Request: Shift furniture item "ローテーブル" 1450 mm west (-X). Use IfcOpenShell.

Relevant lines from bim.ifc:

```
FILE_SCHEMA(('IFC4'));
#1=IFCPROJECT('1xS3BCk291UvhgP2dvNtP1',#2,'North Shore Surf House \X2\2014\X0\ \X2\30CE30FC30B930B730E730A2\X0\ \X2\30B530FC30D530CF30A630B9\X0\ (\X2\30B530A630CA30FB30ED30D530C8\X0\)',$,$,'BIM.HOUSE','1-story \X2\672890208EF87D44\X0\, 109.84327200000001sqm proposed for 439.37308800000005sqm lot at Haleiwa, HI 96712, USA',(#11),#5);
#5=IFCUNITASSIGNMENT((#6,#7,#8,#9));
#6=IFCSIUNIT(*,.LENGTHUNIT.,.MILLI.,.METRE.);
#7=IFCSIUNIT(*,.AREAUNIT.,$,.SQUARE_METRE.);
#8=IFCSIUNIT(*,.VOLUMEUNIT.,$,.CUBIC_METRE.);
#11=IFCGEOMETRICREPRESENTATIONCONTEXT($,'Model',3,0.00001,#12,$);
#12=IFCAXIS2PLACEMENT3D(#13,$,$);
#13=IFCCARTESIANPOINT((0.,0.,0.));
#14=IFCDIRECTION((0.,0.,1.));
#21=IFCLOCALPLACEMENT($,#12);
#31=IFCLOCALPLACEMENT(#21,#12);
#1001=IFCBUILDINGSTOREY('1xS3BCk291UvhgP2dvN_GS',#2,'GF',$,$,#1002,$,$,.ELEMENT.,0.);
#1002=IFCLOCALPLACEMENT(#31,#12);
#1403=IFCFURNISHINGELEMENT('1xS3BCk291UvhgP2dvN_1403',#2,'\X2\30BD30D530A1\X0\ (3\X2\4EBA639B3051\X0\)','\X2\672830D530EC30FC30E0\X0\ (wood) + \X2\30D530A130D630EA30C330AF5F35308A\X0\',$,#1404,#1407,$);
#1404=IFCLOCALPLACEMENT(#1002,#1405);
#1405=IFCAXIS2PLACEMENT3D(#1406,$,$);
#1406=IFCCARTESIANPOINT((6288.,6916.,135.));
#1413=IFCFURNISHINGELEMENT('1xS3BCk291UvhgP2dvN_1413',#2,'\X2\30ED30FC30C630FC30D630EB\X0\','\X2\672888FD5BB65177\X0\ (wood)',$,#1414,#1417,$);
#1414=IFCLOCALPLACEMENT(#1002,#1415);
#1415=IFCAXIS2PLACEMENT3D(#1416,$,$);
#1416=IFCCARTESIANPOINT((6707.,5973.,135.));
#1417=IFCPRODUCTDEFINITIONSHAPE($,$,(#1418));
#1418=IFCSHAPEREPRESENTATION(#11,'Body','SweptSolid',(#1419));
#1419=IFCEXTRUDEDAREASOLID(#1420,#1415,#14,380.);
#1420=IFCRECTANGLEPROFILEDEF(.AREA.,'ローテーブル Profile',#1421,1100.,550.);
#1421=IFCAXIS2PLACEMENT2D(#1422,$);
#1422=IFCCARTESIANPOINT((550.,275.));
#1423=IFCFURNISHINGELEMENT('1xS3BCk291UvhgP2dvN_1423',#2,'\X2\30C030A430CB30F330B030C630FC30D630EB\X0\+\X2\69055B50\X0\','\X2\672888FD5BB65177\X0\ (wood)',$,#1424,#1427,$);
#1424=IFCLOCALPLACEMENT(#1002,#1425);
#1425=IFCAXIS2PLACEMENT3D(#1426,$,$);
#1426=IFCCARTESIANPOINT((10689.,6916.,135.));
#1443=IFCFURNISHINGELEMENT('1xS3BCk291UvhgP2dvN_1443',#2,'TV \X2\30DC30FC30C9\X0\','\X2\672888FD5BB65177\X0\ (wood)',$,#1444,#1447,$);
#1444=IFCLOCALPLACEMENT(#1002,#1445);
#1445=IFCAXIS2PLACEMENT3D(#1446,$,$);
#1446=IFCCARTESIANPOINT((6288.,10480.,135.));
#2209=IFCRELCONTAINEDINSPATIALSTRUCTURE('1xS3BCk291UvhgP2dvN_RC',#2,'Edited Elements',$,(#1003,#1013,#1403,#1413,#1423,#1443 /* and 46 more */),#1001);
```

```python
import ifcopenshell
import ifcopenshell.api.geometry
import ifcopenshell.util.placement
import ifcopenshell.util.unit

model = ifcopenshell.open("bim.ifc")
unit_scale = ifcopenshell.util.unit.calculate_unit_scale(model)

item = model.by_guid("1xS3BCk291UvhgP2dvN_1413")
matrix = ifcopenshell.util.placement.get_local_placement(item.ObjectPlacement)
matrix[0, 3] -= 1.45 / unit_scale
ifcopenshell.api.geometry.edit_object_placement(model, product=item, matrix=matrix, is_si=False)

print(ifcopenshell.util.placement.get_local_placement(item.ObjectPlacement).round(3) + 0.0)

model.write("bim_edited.ifc")
```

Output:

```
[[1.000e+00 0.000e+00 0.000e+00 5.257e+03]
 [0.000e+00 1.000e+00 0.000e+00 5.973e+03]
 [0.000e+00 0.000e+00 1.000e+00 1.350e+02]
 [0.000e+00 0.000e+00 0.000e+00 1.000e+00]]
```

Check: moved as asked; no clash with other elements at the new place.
